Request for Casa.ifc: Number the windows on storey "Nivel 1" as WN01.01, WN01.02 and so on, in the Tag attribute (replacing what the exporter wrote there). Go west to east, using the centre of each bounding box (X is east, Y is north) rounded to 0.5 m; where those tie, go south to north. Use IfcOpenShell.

First a look at what the model holds.

```python
import ifcopenshell
import ifcopenshell.util.element
import ifcopenshell.util.placement

model = ifcopenshell.open("Casa.ifc")
print(model.schema)
storey = next(s for s in model.by_type("IfcBuildingStorey") if s.Name == "Nivel 1")
windows = [e for e in ifcopenshell.util.element.get_decomposition(storey) if e.is_a("IfcWindow")]
for e in sorted(windows, key=lambda e: e.id()):
    origin = ifcopenshell.util.placement.get_local_placement(e.ObjectPlacement)[:3, 3]
    print(e.id(), e.Tag, e.Name, origin.round(2) + 0.0, sep=" | ")
```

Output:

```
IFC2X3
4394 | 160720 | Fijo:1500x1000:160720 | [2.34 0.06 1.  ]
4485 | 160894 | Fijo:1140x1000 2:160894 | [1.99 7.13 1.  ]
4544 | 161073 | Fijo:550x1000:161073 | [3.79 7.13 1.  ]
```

```python
import ifcopenshell
import ifcopenshell.geom
import ifcopenshell.util.element
import ifcopenshell.util.shape

model = ifcopenshell.open("Casa.ifc")
settings = ifcopenshell.geom.settings()
settings.set("use-world-coords", True)


def centre(element):
    shape = ifcopenshell.geom.create_shape(settings, element)
    return ifcopenshell.util.shape.get_bbox_centroid(shape.geometry)


storey = next(s for s in model.by_type("IfcBuildingStorey") if s.Name == "Nivel 1")
windows = [e for e in ifcopenshell.util.element.get_decomposition(storey) if e.is_a("IfcWindow")]

# Insertion points can sit at a corner or the storey origin, so sort by the geometry (in metres).
centres = {e: centre(e) for e in windows}
windows.sort(key=lambda e: (round(centres[e][0] / 0.5), centres[e][1]))

for i, e in enumerate(windows, start=1):
    number = f"WN01.{i:02d}"
    e.Tag = number
    print(e.id(), number)

model.write("Casa_edited.ifc")
```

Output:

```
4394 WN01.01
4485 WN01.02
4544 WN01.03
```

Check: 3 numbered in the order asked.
